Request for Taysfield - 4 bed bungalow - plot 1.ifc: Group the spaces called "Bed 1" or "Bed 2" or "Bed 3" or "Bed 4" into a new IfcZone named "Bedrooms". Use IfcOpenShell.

First a look at what the model holds.

```python
import ifcopenshell

model = ifcopenshell.open("Taysfield - 4 bed bungalow - plot 1.ifc")
print(model.schema)
seen = {}
for space in model.by_type("IfcSpace"):
    seen[space.LongName] = seen.get(space.LongName, 0) + 1
for name, count in sorted(seen.items(), key=str):
    print(count, "x", name)
print("zones:", [z.Name for z in model.by_type("IfcZone")][:20])
```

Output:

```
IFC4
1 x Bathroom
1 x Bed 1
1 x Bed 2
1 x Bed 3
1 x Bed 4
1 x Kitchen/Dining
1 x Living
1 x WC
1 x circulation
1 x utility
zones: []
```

```python
import ifcopenshell
import ifcopenshell.api.group
import ifcopenshell.api.root

model = ifcopenshell.open("Taysfield - 4 bed bungalow - plot 1.ifc")

names = {"Bed 1", "Bed 2", "Bed 3", "Bed 4"}
spaces = [s for s in model.by_type("IfcSpace") if s.LongName in names]

zone = ifcopenshell.api.root.create_entity(model, ifc_class="IfcZone", name="Bedrooms")
ifcopenshell.api.group.assign_group(model, products=spaces, group=zone)
print(len(spaces), "spaces in", zone.Name)

model.write("Taysfield - 4 bed bungalow - plot 1_edited.ifc")
```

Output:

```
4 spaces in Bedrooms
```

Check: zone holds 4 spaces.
